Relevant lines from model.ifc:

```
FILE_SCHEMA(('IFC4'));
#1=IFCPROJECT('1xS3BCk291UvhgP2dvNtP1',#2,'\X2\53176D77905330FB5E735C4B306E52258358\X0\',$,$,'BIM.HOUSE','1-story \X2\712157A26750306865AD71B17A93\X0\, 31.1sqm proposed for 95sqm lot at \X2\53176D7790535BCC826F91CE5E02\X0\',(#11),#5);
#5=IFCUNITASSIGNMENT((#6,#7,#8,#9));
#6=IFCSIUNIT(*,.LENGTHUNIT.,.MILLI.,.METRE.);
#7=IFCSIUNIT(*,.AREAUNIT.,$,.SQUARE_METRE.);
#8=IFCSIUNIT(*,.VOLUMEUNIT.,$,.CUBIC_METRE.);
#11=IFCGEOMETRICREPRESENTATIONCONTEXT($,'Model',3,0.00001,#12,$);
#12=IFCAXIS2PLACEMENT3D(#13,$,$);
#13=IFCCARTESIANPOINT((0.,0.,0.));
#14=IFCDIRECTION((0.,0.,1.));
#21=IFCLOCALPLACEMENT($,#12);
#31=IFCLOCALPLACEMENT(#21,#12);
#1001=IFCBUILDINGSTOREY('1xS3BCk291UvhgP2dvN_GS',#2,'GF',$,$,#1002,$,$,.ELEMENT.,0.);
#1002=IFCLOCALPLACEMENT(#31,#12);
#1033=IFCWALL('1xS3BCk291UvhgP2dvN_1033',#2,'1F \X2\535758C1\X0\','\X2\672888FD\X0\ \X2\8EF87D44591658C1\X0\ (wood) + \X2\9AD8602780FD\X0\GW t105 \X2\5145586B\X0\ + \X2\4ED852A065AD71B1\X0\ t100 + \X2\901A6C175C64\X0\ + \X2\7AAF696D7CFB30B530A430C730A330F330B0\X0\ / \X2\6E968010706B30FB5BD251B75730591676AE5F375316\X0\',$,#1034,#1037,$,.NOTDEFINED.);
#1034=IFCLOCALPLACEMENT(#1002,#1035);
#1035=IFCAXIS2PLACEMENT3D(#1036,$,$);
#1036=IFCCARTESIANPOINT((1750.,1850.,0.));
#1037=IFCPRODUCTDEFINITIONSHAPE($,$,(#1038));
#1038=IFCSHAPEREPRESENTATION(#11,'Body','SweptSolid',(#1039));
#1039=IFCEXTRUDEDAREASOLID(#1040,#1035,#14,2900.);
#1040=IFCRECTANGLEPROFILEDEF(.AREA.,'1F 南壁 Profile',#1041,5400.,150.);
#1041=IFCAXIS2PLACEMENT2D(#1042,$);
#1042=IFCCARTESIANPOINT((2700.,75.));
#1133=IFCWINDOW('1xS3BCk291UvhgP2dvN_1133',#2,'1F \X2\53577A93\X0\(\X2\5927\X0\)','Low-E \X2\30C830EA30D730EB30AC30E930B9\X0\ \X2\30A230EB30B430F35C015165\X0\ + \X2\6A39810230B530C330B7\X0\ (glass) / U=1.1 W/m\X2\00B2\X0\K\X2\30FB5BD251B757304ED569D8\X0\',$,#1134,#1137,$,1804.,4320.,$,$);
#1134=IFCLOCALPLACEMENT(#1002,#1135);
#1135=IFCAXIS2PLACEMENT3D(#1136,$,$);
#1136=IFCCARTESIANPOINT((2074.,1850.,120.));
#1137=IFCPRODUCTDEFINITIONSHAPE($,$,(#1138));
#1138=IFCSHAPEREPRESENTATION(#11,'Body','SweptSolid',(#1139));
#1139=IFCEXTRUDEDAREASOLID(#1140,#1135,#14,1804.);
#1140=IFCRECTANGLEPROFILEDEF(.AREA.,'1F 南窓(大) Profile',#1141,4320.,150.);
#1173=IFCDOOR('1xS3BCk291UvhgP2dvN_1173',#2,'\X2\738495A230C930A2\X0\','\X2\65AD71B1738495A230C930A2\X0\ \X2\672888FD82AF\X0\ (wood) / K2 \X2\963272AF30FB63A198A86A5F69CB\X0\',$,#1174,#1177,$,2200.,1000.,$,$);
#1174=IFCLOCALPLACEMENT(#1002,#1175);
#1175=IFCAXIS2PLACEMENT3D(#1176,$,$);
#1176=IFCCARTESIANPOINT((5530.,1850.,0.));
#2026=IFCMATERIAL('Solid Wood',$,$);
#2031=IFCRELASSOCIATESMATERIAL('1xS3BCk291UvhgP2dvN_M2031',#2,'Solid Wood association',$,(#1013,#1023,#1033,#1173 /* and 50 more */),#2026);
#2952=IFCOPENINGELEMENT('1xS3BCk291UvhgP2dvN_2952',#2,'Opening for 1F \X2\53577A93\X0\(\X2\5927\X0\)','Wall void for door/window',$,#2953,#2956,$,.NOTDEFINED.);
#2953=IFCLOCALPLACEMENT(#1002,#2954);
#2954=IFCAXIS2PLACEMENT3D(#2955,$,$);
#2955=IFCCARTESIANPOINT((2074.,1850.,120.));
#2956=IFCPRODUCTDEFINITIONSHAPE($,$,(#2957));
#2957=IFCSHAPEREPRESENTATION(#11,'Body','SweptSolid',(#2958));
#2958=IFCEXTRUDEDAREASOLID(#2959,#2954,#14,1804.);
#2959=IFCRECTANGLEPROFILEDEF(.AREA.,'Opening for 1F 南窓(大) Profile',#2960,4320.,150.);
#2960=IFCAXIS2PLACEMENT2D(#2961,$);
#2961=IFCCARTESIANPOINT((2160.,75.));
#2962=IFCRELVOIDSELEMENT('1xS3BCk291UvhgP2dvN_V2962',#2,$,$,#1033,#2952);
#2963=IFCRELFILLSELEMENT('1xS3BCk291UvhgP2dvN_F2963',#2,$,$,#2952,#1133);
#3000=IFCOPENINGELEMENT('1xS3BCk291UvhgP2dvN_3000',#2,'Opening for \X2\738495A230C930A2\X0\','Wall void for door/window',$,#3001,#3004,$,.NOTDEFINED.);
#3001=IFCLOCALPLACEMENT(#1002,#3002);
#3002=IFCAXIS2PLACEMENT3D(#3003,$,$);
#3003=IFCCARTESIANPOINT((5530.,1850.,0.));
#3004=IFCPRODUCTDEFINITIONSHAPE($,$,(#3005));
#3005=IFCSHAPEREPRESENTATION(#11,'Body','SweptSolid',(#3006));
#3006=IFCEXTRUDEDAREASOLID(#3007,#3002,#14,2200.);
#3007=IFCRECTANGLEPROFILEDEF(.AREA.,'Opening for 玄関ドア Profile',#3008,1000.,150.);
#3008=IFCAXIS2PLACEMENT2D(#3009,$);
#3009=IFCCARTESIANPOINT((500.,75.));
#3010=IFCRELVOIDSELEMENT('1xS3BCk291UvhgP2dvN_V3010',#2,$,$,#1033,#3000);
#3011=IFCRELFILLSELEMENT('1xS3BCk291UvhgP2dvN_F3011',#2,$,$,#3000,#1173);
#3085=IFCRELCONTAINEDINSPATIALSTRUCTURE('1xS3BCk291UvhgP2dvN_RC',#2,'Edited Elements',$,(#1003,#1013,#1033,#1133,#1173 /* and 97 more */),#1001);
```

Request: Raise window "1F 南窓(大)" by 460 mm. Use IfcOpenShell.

```python
import numpy as np
import ifcopenshell
import ifcopenshell.api.geometry
import ifcopenshell.util.placement
import ifcopenshell.util.unit

model = ifcopenshell.open("model.ifc")
unit_scale = ifcopenshell.util.unit.calculate_unit_scale(model)

window = model.by_id(1133)
opening = window.FillsVoids[0].RelatingOpeningElement
dz = 0.46 / unit_scale

shift = np.array([0.0, 0.0, dz])
# The window is not placed relative to its opening, so move both.
for product in (opening, window):
    matrix = ifcopenshell.util.placement.get_local_placement(product.ObjectPlacement)
    matrix[:3, 3] += shift
    ifcopenshell.api.geometry.edit_object_placement(model, product=product, matrix=matrix, is_si=False)

print(f"moved by {dz * unit_scale:+.3f} m")

model.write("model_edited.ifc")
```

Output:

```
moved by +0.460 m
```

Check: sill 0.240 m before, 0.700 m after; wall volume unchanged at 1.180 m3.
